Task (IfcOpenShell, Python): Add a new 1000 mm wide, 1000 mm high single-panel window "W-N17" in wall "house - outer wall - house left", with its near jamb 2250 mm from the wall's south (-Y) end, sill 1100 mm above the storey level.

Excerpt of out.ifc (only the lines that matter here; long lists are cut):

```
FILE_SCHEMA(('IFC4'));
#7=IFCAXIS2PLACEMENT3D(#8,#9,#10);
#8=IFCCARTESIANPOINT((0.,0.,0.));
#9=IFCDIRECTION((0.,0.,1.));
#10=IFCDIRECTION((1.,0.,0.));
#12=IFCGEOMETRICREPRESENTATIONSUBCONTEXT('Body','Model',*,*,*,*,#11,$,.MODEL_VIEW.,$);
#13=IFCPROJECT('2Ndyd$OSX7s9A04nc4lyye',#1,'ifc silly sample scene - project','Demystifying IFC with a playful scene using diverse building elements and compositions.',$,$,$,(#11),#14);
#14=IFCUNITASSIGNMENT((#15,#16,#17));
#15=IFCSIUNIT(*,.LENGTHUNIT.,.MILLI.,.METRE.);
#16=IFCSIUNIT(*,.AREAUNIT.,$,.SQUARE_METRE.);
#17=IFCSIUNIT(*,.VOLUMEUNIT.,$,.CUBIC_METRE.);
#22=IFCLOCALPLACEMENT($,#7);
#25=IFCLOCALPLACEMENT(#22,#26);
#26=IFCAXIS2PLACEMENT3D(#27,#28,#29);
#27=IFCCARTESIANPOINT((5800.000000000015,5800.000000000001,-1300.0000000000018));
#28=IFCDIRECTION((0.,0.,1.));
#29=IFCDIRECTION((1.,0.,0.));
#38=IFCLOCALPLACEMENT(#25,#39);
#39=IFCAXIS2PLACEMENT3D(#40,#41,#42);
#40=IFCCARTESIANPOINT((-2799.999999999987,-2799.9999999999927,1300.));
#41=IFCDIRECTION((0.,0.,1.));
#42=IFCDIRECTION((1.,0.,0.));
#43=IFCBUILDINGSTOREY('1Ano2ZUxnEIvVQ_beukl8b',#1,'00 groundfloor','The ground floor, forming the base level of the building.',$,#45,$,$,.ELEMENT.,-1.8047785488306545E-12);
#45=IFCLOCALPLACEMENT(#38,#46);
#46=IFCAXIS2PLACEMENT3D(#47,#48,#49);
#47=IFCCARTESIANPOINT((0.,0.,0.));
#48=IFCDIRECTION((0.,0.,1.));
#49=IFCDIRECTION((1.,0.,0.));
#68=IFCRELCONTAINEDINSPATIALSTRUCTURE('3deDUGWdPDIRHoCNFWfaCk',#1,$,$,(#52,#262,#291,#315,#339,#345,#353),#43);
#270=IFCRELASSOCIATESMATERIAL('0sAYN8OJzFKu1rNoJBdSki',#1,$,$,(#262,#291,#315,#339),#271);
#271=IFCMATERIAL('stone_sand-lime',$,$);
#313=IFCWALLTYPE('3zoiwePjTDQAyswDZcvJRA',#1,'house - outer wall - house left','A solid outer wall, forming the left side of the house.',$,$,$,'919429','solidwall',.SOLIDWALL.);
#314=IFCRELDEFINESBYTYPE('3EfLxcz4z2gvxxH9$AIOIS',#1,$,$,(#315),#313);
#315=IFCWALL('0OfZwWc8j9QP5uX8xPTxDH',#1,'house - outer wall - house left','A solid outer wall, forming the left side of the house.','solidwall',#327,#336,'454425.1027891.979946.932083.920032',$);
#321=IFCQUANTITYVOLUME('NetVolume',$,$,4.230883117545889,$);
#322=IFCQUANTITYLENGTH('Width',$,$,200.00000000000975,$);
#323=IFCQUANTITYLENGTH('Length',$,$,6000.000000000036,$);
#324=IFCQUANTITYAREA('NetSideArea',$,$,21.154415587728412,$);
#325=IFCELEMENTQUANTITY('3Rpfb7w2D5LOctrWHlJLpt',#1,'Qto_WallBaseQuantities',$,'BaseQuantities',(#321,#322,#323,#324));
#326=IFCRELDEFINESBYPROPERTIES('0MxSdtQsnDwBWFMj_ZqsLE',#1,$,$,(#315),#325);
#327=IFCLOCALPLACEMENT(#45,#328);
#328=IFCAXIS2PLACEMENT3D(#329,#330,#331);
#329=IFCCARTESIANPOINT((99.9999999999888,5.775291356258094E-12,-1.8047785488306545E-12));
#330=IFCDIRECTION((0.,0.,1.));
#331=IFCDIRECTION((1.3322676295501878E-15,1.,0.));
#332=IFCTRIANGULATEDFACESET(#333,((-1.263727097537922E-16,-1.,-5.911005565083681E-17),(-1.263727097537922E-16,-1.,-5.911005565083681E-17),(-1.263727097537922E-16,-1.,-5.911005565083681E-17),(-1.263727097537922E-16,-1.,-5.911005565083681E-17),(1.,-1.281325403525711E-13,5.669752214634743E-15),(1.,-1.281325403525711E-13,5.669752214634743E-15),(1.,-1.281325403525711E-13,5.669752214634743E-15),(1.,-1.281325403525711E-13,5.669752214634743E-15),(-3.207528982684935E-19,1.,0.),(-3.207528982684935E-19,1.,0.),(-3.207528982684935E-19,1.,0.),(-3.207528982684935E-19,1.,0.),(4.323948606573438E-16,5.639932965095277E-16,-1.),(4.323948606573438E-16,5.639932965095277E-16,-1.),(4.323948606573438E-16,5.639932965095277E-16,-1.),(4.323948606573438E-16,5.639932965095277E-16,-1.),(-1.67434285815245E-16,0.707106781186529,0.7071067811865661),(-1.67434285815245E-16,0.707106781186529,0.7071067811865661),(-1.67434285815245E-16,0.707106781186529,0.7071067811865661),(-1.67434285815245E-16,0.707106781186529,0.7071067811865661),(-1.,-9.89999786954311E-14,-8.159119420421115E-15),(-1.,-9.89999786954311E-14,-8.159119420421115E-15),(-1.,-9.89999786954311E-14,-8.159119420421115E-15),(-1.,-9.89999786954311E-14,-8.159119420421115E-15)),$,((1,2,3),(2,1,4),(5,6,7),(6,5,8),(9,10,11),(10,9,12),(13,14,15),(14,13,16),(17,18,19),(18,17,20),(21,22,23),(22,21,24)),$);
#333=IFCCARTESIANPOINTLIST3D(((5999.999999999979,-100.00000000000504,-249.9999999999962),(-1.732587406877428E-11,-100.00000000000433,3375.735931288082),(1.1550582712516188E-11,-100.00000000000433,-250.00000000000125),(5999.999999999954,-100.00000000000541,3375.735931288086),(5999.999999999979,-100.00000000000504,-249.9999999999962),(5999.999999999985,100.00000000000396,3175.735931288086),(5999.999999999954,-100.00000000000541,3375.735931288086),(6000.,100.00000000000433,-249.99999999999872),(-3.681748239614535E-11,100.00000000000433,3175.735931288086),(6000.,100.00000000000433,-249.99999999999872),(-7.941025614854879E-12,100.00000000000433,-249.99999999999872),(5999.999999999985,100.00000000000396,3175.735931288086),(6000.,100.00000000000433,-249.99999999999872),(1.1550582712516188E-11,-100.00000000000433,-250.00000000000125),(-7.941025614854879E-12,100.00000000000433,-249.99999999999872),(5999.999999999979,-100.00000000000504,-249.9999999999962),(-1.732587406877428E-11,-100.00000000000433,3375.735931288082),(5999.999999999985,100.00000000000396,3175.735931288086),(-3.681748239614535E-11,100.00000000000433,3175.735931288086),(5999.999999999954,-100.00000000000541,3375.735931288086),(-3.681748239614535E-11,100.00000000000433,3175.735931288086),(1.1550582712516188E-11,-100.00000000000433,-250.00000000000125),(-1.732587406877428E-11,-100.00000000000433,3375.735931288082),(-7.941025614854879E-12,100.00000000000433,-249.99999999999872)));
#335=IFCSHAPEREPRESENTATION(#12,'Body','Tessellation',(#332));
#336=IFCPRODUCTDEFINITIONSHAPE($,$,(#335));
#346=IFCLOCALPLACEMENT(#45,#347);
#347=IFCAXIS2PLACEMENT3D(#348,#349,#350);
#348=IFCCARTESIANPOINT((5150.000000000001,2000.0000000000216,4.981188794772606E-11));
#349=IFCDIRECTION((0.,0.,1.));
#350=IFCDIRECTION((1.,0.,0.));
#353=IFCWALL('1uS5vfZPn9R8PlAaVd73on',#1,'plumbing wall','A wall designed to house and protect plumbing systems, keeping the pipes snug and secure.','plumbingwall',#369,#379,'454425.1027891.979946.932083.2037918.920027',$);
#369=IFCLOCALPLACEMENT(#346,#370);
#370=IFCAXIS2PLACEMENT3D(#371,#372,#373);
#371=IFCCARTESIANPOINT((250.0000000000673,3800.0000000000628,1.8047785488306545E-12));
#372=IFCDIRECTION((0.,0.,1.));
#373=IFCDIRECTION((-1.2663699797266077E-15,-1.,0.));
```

```python
import numpy as np
import ifcopenshell
import ifcopenshell.api.feature
import ifcopenshell.api.geometry
import ifcopenshell.api.pset
import ifcopenshell.api.root
import ifcopenshell.api.spatial
import ifcopenshell.geom
import ifcopenshell.util.element
import ifcopenshell.util.placement
import ifcopenshell.util.representation
import ifcopenshell.util.shape
import ifcopenshell.util.unit

model = ifcopenshell.open("out.ifc")
unit_scale = ifcopenshell.util.unit.calculate_unit_scale(model)
area_scale = ifcopenshell.util.unit.calculate_unit_scale(model, "AREAUNIT")
volume_scale = ifcopenshell.util.unit.calculate_unit_scale(model, "VOLUMEUNIT")
settings = ifcopenshell.geom.settings()


def volume(element):
    """Net volume in cubic metres, openings subtracted."""
    shape = ifcopenshell.geom.create_shape(settings, element)
    return ifcopenshell.util.shape.get_volume(shape.geometry)


wall = model.by_guid("0OfZwWc8j9QP5uX8xPTxDH")
storey = ifcopenshell.util.element.get_container(wall, ifc_class="IfcBuildingStorey")
context = ifcopenshell.util.representation.get_context(model, "Model", "Body", "MODEL_VIEW")
before = volume(wall)

width, height, from_end, sill = 1, 1, 2.25, 1.1  # metres

# The wall runs along its own X axis, and the end named is its -X end.
wall_shape = ifcopenshell.geom.create_shape(settings, wall)
x, y, z = ifcopenshell.util.shape.get_vertices(wall_shape.geometry).T
start = x.min() + from_end
face, thickness = float(y.min()), float(y.max() - y.min())
wall_matrix = ifcopenshell.util.placement.get_local_placement(wall.ObjectPlacement)
level = ifcopenshell.util.placement.get_local_placement(storey.ObjectPlacement)[2, 3]


def in_wall(x, y):
    """Placement at x, y metres in the wall's axes, at sill height."""
    matrix = wall_matrix.copy()
    matrix[:, 3] = wall_matrix @ np.array([x / unit_scale, y / unit_scale, 0.0, 1.0])
    matrix[2, 3] = level + sill / unit_scale
    return matrix


# Opening: a box that overshoots both wall faces by 50 mm.
opening = ifcopenshell.api.root.create_entity(model, ifc_class="IfcOpeningElement", predefined_type="OPENING")
box = ifcopenshell.api.geometry.add_wall_representation(
    model, context=context, length=width, height=height, thickness=thickness + 0.1
)
ifcopenshell.api.geometry.assign_representation(model, product=opening, representation=box)
ifcopenshell.api.geometry.edit_object_placement(model, product=opening, matrix=in_wall(start, face - 0.05), is_si=False)
ifcopenshell.api.feature.add_feature(model, feature=opening, element=wall)

window = ifcopenshell.api.root.create_entity(model, ifc_class="IfcWindow", name="W-N17", predefined_type="WINDOW")
window.OverallWidth, window.OverallHeight = width / unit_scale, height / unit_scale
window.PartitioningType = "SINGLE_PANEL"
body = ifcopenshell.api.geometry.add_window_representation(
    model,
    context=context,
    overall_width=window.OverallWidth,
    overall_height=window.OverallHeight,
    partition_type="SINGLE_PANEL",
)
ifcopenshell.api.geometry.assign_representation(model, product=window, representation=body)
ifcopenshell.api.spatial.assign_container(model, products=[window], relating_structure=storey)
ifcopenshell.api.feature.add_filling(model, opening=opening, element=window)

# Centre the window in the wall's thickness.
ifcopenshell.api.geometry.edit_object_placement(model, product=window, matrix=in_wall(start, face), is_si=False)
window_shape = ifcopenshell.geom.create_shape(settings, window)
depth = ifcopenshell.util.shape.get_vertices(window_shape.geometry)[:, 1]
offset = face + thickness / 2 - (depth.min() + depth.max()) / 2
ifcopenshell.api.geometry.edit_object_placement(model, product=window, matrix=in_wall(start, offset), is_si=False)

after = volume(wall)

# Update the wall's stored quantities.
qto = model.by_id(ifcopenshell.util.element.get_pset(wall, "Qto_WallBaseQuantities", should_inherit=False)["id"])
ifcopenshell.api.pset.edit_qto(model, qto=qto, properties={
    "NetVolume": after / volume_scale,
    "NetSideArea": after / thickness / area_scale,
})

print(f"wall volume {before:.3f} -> {after:.3f} m3")

model.write("out_updated.ifc")
```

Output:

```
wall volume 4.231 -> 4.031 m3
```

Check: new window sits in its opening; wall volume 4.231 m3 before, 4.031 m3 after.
